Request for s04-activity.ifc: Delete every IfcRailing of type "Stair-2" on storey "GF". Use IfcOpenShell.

First a look at what the model holds.

```python
import ifcopenshell
import ifcopenshell.util.element

model = ifcopenshell.open("s04-activity.ifc")
print(model.schema)
storey = next(s for s in model.by_type("IfcBuildingStorey") if s.Name == "GF")
railings = [e for e in ifcopenshell.util.element.get_decomposition(storey) if e.is_a("IfcRailing")]
seen = {}
for e in railings:
    element_type = ifcopenshell.util.element.get_type(e)
    name = element_type.Name if element_type not in (None, e) else None
    seen[name] = seen.get(name, 0) + 1
for name, count in sorted(seen.items(), key=str):
    print(count, "x", name)
```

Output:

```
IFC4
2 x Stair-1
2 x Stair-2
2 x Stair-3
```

```python
import ifcopenshell
import ifcopenshell.api.root
import ifcopenshell.util.element

model = ifcopenshell.open("s04-activity.ifc")

storey = next(s for s in model.by_type("IfcBuildingStorey") if s.Name == "GF")
railings = [e for e in ifcopenshell.util.element.get_decomposition(storey) if e.is_a("IfcRailing")]
targets = [e for e in railings if (t := ifcopenshell.util.element.get_type(e)) not in (None, e) and t.Name == "Stair-2"]

for e in targets:
    ifcopenshell.api.root.remove_product(model, product=e)
print(len(targets), "removed")

model.write("s04-activity_edited.ifc")
```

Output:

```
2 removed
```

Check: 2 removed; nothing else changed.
